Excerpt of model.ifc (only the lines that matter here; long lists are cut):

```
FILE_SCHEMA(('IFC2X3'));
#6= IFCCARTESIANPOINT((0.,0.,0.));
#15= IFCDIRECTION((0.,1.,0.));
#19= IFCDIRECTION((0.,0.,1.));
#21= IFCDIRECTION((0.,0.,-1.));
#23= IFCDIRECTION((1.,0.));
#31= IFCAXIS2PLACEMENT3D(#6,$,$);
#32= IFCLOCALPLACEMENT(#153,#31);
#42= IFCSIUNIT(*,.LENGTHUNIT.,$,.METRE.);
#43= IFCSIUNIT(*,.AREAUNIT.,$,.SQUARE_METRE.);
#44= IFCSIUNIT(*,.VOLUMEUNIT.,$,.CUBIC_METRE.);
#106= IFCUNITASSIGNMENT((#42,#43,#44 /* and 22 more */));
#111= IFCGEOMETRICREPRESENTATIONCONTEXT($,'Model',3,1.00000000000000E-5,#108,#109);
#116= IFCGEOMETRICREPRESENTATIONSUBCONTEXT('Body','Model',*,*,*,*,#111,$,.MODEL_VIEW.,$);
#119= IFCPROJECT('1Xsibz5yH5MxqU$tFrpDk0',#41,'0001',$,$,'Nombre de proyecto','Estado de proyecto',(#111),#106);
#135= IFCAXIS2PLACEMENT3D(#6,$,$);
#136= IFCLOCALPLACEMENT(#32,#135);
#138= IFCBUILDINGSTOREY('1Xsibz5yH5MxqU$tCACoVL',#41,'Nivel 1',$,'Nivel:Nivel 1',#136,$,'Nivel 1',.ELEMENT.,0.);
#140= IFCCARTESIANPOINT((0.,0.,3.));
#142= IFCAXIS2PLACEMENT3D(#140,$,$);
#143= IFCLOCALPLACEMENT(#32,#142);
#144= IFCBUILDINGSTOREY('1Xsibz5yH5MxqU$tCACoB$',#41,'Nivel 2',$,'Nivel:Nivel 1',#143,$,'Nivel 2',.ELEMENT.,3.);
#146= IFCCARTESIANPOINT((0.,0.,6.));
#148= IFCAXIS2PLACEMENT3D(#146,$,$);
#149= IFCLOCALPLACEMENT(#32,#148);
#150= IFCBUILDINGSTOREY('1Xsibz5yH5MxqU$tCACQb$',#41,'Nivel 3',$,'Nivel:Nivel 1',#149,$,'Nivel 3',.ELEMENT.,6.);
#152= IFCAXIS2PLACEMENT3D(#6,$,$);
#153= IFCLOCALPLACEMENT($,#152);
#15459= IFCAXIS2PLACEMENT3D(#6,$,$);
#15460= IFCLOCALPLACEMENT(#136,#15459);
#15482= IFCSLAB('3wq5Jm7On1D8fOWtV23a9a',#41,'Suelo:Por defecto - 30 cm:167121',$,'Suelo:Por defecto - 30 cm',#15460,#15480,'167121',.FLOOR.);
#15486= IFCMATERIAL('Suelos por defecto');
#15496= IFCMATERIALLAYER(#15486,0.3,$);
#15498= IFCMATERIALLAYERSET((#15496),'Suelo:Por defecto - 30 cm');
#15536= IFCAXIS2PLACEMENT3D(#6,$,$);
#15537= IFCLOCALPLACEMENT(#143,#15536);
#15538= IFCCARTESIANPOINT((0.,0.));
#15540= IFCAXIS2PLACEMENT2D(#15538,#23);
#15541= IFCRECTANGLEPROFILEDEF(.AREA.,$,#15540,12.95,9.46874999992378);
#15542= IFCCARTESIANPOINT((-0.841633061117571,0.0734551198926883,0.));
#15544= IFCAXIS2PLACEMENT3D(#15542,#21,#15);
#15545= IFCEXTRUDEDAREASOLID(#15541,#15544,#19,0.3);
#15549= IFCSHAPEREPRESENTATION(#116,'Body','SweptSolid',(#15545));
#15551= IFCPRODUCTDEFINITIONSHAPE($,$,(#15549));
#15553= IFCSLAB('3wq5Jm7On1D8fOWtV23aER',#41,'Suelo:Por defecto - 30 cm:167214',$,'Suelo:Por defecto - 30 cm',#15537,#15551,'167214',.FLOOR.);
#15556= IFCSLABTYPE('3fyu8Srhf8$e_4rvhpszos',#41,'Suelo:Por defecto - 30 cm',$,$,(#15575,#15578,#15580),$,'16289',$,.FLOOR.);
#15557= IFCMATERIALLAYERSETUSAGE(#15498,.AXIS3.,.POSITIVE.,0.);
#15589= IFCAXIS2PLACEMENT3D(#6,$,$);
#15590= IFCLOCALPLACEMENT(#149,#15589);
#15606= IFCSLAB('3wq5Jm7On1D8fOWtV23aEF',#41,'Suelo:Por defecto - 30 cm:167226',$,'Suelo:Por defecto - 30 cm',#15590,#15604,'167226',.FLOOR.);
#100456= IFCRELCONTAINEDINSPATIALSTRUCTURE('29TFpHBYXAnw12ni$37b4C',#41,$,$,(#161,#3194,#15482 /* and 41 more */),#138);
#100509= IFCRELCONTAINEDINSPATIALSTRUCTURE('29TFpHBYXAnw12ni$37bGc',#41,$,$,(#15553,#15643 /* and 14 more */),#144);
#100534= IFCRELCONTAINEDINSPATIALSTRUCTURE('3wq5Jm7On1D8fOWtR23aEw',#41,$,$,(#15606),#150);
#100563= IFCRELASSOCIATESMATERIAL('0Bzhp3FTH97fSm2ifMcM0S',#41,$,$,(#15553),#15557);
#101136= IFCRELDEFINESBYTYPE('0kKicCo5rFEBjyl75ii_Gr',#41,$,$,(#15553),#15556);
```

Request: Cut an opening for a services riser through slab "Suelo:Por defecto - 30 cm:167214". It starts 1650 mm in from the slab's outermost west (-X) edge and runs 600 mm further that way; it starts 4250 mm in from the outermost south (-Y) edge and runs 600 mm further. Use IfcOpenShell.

```python
import numpy as np
import ifcopenshell
import ifcopenshell.api.feature
import ifcopenshell.api.geometry
import ifcopenshell.api.root
import ifcopenshell.geom
import ifcopenshell.util.placement
import ifcopenshell.util.representation
import ifcopenshell.util.shape
import ifcopenshell.util.unit

model = ifcopenshell.open("model.ifc")
unit_scale = ifcopenshell.util.unit.calculate_unit_scale(model)
settings = ifcopenshell.geom.settings()


def volume(element):
    """Net volume in cubic metres, openings subtracted."""
    shape = ifcopenshell.geom.create_shape(settings, element)
    return ifcopenshell.util.shape.get_volume(shape.geometry)


slab = model.by_guid("3wq5Jm7On1D8fOWtV23aER")
before = volume(slab)

# Extent in the slab's own axes, in metres. The edges named are its -X and -Y sides.
slab_shape = ifcopenshell.geom.create_shape(settings, slab)
vertices = ifcopenshell.util.shape.get_vertices(slab_shape.geometry)
x_min, y_min, bottom = vertices.min(axis=0)
top = vertices[:, 2].max()

opening = ifcopenshell.api.root.create_entity(model, ifc_class="IfcOpeningElement", name="Services riser opening")
context = ifcopenshell.util.representation.get_context(model, "Model", "Body", "MODEL_VIEW")
width, depth = 0.6, 0.6
outline = [(0.0, 0.0), (width, 0.0), (width, depth), (0.0, depth), (0.0, 0.0)]
# Overshoot both faces by 50 mm so the cut is clean.
shape = ifcopenshell.api.geometry.add_slab_representation(
    model, context=context, depth=top - bottom + 0.1, polyline=outline
)
ifcopenshell.api.geometry.assign_representation(model, product=opening, representation=shape)

matrix = ifcopenshell.util.placement.get_local_placement(slab.ObjectPlacement)
matrix[:, 3] = matrix @ np.append(np.array([x_min + 1.65, y_min + 4.25, bottom - 0.05]) / unit_scale, 1.0)
ifcopenshell.api.geometry.edit_object_placement(model, product=opening, matrix=matrix, is_si=False)
ifcopenshell.api.feature.add_feature(model, feature=opening, element=slab)

after = volume(slab)

print(f"slab volume {before:.3f} -> {after:.3f} m3")

model.write("model_rev.ifc")
```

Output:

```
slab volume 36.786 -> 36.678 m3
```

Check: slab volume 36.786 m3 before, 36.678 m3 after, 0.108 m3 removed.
